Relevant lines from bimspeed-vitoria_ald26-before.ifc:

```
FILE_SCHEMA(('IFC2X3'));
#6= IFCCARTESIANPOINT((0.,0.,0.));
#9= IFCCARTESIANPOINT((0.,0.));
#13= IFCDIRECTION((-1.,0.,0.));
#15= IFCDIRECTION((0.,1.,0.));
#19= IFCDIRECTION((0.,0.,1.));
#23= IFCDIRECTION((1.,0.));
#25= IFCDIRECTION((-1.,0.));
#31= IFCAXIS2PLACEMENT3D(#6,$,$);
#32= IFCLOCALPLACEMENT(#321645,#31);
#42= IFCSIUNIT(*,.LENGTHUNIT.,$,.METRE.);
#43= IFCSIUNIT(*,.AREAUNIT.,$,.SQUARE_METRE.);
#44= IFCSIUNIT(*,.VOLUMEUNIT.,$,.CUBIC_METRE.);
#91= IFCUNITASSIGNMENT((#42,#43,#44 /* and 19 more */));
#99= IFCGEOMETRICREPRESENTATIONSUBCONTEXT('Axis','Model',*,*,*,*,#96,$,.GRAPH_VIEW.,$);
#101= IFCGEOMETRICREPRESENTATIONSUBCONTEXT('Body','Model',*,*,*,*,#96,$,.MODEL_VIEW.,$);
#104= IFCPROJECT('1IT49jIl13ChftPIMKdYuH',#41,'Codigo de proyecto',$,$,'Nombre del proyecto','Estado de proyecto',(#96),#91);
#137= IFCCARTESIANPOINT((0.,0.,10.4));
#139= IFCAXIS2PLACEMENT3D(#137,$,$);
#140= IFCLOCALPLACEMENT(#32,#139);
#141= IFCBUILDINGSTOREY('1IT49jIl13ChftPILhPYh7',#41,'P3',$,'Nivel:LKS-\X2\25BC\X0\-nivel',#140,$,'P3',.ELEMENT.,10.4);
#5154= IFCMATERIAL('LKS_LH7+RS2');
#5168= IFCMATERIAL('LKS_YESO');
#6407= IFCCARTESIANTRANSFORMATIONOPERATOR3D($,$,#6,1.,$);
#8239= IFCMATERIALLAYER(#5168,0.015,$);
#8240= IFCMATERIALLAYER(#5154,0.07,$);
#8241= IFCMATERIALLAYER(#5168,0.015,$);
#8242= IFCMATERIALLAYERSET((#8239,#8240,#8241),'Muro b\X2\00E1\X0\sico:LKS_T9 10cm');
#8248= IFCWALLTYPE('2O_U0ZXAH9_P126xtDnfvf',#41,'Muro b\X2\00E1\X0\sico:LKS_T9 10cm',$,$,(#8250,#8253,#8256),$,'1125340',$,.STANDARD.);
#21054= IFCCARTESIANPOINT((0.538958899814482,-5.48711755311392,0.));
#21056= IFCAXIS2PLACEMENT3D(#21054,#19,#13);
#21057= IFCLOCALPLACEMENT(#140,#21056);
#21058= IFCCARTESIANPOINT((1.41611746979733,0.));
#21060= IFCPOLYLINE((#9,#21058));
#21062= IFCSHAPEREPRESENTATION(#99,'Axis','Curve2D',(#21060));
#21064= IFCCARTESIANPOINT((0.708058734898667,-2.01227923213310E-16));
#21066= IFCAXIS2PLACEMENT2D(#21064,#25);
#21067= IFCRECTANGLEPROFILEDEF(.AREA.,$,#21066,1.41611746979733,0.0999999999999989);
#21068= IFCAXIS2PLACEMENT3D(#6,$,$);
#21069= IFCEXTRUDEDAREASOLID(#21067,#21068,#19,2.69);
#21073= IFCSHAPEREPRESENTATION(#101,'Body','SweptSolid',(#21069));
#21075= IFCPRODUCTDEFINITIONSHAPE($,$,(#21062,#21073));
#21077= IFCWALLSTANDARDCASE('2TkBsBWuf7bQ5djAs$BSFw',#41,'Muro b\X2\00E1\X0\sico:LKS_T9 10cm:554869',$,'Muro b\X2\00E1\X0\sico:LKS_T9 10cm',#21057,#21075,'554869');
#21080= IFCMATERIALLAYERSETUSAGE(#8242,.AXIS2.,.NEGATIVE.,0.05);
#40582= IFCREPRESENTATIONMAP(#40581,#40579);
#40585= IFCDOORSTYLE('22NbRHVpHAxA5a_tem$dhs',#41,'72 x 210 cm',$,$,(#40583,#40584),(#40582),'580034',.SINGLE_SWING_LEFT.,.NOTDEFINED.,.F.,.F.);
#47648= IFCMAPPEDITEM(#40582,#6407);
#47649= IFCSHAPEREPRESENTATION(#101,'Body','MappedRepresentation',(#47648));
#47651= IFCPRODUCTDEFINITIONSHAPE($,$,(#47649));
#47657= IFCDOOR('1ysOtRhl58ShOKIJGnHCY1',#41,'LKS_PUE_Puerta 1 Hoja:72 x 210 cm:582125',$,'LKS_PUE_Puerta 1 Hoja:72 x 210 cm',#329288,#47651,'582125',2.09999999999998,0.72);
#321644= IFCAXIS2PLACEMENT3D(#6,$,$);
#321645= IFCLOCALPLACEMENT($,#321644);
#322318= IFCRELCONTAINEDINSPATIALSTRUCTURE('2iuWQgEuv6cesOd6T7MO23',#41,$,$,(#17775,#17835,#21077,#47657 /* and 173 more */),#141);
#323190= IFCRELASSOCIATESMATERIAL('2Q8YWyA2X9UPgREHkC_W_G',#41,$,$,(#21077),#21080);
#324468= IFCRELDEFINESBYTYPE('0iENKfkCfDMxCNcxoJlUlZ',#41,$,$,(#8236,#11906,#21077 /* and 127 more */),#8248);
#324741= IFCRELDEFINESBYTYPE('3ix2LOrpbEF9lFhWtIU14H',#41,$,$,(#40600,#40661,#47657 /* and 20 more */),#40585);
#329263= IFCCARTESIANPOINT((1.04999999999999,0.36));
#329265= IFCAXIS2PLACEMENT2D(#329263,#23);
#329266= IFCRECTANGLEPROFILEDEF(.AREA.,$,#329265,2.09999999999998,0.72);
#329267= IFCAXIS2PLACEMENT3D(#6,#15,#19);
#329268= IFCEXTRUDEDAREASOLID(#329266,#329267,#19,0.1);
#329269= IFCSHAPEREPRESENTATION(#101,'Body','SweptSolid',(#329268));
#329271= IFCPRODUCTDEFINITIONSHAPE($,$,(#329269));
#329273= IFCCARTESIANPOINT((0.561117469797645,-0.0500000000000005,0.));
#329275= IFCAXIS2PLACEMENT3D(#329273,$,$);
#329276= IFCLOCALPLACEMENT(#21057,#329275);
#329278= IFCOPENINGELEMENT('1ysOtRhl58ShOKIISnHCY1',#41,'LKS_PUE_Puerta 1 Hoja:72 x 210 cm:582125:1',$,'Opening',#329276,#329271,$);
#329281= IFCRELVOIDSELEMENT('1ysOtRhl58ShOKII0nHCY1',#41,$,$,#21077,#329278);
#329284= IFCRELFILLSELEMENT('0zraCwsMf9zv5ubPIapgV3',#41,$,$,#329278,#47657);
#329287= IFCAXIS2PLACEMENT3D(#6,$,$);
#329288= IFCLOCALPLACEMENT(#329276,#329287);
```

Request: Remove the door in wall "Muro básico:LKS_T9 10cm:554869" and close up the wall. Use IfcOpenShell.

```python
import ifcopenshell
import ifcopenshell.api.feature
import ifcopenshell.api.root
import ifcopenshell.geom
import ifcopenshell.util.shape

model = ifcopenshell.open("bimspeed-vitoria_ald26-before.ifc")
settings = ifcopenshell.geom.settings()


def volume(element):
    """Net volume in cubic metres, openings subtracted."""
    shape = ifcopenshell.geom.create_shape(settings, element)
    return ifcopenshell.util.shape.get_volume(shape.geometry)


door = model.by_guid("1ysOtRhl58ShOKIJGnHCY1")
opening = door.FillsVoids[0].RelatingOpeningElement
wall = opening.VoidsElements[0].RelatingBuildingElement
before = volume(wall)

ifcopenshell.api.root.remove_product(model, product=door)
ifcopenshell.api.feature.remove_feature(model, feature=opening)

after = volume(wall)

print(f"wall volume {before:.3f} -> {after:.3f} m3")

model.write("bimspeed-vitoria_ald26-before_v2.ifc")
```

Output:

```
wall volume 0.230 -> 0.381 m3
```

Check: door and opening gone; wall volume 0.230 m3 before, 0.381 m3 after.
